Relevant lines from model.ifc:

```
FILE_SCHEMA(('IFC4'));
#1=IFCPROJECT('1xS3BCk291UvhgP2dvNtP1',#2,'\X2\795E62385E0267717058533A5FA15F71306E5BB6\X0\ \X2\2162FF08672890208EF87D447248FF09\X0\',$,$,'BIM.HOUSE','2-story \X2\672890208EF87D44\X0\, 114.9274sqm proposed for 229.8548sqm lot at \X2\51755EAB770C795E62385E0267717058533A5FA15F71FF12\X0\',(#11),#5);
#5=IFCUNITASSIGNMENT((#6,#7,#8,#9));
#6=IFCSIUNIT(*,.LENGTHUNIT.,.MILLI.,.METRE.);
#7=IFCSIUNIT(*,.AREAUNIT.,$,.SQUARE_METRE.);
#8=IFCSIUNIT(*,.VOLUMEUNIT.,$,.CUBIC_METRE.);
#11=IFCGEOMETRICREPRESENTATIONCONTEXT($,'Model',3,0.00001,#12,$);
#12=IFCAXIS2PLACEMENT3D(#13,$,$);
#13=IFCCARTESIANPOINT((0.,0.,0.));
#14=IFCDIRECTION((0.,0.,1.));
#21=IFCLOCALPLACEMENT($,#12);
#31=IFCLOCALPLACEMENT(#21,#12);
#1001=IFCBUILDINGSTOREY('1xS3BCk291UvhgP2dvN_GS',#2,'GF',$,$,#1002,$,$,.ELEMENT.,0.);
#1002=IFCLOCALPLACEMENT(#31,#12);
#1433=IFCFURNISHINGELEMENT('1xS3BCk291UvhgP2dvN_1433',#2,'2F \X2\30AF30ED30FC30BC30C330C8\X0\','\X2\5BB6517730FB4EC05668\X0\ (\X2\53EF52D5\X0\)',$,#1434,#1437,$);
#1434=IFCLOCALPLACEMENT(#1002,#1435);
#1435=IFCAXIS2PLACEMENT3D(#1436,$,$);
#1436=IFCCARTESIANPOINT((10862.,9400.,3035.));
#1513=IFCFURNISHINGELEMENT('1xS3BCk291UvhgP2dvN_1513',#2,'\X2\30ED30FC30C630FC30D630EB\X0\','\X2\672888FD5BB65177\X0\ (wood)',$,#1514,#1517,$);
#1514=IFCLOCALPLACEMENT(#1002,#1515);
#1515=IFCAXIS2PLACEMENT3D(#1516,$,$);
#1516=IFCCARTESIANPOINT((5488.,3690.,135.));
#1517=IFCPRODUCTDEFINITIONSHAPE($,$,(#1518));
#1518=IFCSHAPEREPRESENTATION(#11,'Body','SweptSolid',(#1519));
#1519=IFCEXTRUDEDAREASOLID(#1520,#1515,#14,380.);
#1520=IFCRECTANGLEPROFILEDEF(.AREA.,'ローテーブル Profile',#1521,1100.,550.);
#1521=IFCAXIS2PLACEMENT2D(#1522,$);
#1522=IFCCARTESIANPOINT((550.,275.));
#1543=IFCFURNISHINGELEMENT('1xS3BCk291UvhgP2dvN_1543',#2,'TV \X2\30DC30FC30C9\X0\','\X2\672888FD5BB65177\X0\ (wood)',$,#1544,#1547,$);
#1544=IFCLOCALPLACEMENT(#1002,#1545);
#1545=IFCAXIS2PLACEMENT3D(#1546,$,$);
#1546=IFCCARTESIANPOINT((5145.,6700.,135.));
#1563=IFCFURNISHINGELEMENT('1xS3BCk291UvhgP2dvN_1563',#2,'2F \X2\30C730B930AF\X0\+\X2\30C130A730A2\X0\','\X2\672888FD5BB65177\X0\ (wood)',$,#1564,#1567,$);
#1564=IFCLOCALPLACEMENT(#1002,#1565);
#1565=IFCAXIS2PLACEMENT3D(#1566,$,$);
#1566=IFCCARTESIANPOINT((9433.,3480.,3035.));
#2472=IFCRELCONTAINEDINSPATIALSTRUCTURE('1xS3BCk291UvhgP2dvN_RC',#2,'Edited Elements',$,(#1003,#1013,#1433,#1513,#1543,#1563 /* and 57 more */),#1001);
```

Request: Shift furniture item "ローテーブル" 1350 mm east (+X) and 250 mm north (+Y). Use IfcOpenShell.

```python
import ifcopenshell
import ifcopenshell.api.geometry
import ifcopenshell.util.placement
import ifcopenshell.util.unit

model = ifcopenshell.open("model.ifc")
unit_scale = ifcopenshell.util.unit.calculate_unit_scale(model)

item = model.by_id(1513)
matrix = ifcopenshell.util.placement.get_local_placement(item.ObjectPlacement)
matrix[0, 3] += 1.35 / unit_scale
matrix[1, 3] += 0.25 / unit_scale
ifcopenshell.api.geometry.edit_object_placement(model, product=item, matrix=matrix, is_si=False)

print(ifcopenshell.util.placement.get_local_placement(item.ObjectPlacement).round(3) + 0.0)

model.write("model_v2.ifc")
```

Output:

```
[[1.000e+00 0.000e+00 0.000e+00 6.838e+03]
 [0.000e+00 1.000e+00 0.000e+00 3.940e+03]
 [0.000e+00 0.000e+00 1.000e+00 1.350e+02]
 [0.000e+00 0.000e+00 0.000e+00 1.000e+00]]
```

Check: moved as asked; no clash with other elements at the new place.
